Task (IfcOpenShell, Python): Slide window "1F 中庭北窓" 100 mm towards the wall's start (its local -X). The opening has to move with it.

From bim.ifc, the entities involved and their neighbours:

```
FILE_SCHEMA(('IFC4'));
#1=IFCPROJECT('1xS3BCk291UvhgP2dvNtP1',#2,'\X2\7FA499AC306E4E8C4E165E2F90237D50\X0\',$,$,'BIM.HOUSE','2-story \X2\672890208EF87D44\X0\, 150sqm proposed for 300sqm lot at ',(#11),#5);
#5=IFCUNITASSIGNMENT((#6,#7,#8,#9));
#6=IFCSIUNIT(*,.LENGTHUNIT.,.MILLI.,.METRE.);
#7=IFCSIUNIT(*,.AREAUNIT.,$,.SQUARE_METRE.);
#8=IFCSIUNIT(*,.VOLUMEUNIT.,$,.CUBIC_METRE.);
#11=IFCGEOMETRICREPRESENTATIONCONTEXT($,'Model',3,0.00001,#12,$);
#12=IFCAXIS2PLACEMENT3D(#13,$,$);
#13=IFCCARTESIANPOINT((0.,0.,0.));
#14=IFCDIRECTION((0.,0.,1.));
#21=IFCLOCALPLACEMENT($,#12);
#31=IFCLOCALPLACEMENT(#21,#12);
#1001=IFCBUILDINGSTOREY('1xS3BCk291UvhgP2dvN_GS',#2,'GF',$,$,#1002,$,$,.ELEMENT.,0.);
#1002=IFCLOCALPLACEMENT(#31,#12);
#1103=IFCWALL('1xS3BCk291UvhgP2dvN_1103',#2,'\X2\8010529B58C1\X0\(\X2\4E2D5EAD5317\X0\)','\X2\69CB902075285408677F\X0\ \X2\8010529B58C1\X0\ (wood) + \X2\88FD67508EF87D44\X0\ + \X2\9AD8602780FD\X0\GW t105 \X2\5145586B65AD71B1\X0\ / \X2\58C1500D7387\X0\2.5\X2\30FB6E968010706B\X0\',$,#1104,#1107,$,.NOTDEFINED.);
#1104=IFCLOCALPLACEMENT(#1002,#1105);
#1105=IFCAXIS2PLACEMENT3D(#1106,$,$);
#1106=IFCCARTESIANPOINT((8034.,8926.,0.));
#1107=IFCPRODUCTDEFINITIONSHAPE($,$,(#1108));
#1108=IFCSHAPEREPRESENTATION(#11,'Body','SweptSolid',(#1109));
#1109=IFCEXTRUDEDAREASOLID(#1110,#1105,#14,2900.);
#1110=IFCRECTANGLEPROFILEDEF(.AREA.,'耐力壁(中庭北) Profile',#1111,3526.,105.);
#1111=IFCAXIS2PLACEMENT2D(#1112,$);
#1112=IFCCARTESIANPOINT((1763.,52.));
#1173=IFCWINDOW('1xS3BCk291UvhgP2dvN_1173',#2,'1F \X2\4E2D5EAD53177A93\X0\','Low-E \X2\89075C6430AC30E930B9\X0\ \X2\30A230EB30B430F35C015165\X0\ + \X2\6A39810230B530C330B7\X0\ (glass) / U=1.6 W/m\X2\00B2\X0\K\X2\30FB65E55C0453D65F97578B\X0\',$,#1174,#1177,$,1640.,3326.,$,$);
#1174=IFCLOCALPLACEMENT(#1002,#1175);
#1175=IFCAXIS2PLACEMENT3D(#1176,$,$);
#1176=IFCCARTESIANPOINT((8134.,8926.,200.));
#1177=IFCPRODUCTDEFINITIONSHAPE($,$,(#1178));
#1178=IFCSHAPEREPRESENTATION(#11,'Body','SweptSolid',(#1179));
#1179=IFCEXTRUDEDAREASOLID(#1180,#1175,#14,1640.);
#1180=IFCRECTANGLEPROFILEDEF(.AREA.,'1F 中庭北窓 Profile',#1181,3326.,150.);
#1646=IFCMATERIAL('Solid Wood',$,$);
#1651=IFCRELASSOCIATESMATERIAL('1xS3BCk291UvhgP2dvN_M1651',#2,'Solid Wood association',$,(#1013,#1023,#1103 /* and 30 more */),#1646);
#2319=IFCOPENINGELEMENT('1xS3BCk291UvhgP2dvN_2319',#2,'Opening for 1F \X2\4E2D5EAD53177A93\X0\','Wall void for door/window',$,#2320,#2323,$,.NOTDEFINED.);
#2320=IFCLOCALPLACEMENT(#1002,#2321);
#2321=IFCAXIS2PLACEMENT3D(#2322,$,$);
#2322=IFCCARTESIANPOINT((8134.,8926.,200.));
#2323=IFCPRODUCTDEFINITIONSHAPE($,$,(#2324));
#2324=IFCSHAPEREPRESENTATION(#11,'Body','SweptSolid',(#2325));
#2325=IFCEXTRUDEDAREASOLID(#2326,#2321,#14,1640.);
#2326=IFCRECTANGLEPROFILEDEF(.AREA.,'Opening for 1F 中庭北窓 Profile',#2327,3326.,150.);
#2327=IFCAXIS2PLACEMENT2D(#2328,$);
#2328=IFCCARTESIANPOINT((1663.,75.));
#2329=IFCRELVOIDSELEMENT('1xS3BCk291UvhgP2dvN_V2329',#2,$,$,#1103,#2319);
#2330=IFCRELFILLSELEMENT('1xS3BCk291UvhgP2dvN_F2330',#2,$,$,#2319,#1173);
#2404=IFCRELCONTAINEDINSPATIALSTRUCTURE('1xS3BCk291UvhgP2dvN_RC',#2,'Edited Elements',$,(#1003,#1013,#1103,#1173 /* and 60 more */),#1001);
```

```python
import ifcopenshell
import ifcopenshell.api.geometry
import ifcopenshell.util.placement
import ifcopenshell.util.unit

model = ifcopenshell.open("bim.ifc")
unit_scale = ifcopenshell.util.unit.calculate_unit_scale(model)

window = model.by_id(1173)
opening = window.FillsVoids[0].RelatingOpeningElement
wall = opening.VoidsElements[0].RelatingBuildingElement

wall_matrix = ifcopenshell.util.placement.get_local_placement(wall.ObjectPlacement)
shift = wall_matrix[:3, 0] * -0.1 / unit_scale
before = ifcopenshell.util.placement.get_local_placement(window.ObjectPlacement)[:3, 3].copy()

# The window is not placed relative to its opening, so move both.
for product in (opening, window):
    matrix = ifcopenshell.util.placement.get_local_placement(product.ObjectPlacement)
    matrix[:3, 3] += shift
    ifcopenshell.api.geometry.edit_object_placement(model, product=product, matrix=matrix, is_si=False)

after = ifcopenshell.util.placement.get_local_placement(window.ObjectPlacement)[:3, 3]
print("window moved by", (after - before).round(3) + 0.0)

model.write("bim_updated.ifc")
```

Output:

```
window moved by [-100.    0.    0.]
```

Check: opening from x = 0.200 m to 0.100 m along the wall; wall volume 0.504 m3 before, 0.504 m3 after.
